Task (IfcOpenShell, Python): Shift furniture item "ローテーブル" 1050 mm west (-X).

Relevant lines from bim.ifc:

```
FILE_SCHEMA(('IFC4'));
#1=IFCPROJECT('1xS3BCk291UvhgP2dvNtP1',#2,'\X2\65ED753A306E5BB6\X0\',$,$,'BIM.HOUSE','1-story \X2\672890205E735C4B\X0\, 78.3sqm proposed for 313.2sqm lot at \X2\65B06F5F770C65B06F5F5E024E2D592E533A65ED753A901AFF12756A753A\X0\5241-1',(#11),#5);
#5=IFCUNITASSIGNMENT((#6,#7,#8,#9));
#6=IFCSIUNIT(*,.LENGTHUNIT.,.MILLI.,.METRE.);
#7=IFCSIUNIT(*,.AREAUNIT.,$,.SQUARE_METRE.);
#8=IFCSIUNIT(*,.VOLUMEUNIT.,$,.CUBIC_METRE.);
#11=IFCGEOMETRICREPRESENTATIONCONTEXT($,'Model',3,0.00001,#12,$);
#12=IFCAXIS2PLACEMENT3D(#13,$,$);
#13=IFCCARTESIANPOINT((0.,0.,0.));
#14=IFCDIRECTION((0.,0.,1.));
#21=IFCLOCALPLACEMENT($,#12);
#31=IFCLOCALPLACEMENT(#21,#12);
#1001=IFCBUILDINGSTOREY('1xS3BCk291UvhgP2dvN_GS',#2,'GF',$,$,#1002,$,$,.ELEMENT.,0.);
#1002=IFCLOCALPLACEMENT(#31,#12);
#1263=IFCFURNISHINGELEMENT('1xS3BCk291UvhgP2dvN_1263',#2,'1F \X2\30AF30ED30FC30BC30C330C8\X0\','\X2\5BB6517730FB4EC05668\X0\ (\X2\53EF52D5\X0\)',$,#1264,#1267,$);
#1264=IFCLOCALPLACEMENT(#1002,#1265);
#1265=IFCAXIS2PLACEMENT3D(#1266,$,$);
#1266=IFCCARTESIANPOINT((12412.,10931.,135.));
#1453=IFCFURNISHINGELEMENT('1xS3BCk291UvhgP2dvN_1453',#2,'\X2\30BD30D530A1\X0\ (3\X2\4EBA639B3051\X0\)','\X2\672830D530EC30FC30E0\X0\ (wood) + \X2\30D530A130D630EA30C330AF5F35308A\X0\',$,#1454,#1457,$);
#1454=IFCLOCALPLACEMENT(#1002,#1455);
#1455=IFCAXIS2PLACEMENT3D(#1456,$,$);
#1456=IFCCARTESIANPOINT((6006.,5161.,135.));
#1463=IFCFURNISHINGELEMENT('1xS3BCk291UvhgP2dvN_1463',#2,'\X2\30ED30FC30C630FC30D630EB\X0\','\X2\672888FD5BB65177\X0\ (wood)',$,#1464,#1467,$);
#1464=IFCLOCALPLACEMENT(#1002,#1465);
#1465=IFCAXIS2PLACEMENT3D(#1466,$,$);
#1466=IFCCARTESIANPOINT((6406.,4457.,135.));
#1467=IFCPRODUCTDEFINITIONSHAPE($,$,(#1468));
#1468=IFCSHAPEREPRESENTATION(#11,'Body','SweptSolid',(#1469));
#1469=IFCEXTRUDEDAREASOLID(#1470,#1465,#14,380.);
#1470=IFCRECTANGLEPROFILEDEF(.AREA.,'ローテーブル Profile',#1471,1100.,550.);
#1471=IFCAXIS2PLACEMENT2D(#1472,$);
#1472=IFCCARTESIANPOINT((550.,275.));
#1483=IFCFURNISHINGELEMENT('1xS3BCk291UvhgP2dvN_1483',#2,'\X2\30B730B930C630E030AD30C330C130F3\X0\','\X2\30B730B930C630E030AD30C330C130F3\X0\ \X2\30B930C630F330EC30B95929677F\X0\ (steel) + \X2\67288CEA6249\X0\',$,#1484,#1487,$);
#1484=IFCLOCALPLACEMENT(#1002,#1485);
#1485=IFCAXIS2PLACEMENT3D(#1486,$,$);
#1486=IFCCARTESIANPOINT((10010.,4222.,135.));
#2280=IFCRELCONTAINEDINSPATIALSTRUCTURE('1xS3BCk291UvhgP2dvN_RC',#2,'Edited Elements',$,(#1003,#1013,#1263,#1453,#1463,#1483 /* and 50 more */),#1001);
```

```python
import ifcopenshell
import ifcopenshell.api.geometry
import ifcopenshell.util.placement
import ifcopenshell.util.unit

model = ifcopenshell.open("bim.ifc")
unit_scale = ifcopenshell.util.unit.calculate_unit_scale(model)

item = model.by_guid("1xS3BCk291UvhgP2dvN_1463")
matrix = ifcopenshell.util.placement.get_local_placement(item.ObjectPlacement)
matrix[0, 3] -= 1.05 / unit_scale
ifcopenshell.api.geometry.edit_object_placement(model, product=item, matrix=matrix, is_si=False)

print(ifcopenshell.util.placement.get_local_placement(item.ObjectPlacement).round(3) + 0.0)

model.write("bim-out.ifc")
```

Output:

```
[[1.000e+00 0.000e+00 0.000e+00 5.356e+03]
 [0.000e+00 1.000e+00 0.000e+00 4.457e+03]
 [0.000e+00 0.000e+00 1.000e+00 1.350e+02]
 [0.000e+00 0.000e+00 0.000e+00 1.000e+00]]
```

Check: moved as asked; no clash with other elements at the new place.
